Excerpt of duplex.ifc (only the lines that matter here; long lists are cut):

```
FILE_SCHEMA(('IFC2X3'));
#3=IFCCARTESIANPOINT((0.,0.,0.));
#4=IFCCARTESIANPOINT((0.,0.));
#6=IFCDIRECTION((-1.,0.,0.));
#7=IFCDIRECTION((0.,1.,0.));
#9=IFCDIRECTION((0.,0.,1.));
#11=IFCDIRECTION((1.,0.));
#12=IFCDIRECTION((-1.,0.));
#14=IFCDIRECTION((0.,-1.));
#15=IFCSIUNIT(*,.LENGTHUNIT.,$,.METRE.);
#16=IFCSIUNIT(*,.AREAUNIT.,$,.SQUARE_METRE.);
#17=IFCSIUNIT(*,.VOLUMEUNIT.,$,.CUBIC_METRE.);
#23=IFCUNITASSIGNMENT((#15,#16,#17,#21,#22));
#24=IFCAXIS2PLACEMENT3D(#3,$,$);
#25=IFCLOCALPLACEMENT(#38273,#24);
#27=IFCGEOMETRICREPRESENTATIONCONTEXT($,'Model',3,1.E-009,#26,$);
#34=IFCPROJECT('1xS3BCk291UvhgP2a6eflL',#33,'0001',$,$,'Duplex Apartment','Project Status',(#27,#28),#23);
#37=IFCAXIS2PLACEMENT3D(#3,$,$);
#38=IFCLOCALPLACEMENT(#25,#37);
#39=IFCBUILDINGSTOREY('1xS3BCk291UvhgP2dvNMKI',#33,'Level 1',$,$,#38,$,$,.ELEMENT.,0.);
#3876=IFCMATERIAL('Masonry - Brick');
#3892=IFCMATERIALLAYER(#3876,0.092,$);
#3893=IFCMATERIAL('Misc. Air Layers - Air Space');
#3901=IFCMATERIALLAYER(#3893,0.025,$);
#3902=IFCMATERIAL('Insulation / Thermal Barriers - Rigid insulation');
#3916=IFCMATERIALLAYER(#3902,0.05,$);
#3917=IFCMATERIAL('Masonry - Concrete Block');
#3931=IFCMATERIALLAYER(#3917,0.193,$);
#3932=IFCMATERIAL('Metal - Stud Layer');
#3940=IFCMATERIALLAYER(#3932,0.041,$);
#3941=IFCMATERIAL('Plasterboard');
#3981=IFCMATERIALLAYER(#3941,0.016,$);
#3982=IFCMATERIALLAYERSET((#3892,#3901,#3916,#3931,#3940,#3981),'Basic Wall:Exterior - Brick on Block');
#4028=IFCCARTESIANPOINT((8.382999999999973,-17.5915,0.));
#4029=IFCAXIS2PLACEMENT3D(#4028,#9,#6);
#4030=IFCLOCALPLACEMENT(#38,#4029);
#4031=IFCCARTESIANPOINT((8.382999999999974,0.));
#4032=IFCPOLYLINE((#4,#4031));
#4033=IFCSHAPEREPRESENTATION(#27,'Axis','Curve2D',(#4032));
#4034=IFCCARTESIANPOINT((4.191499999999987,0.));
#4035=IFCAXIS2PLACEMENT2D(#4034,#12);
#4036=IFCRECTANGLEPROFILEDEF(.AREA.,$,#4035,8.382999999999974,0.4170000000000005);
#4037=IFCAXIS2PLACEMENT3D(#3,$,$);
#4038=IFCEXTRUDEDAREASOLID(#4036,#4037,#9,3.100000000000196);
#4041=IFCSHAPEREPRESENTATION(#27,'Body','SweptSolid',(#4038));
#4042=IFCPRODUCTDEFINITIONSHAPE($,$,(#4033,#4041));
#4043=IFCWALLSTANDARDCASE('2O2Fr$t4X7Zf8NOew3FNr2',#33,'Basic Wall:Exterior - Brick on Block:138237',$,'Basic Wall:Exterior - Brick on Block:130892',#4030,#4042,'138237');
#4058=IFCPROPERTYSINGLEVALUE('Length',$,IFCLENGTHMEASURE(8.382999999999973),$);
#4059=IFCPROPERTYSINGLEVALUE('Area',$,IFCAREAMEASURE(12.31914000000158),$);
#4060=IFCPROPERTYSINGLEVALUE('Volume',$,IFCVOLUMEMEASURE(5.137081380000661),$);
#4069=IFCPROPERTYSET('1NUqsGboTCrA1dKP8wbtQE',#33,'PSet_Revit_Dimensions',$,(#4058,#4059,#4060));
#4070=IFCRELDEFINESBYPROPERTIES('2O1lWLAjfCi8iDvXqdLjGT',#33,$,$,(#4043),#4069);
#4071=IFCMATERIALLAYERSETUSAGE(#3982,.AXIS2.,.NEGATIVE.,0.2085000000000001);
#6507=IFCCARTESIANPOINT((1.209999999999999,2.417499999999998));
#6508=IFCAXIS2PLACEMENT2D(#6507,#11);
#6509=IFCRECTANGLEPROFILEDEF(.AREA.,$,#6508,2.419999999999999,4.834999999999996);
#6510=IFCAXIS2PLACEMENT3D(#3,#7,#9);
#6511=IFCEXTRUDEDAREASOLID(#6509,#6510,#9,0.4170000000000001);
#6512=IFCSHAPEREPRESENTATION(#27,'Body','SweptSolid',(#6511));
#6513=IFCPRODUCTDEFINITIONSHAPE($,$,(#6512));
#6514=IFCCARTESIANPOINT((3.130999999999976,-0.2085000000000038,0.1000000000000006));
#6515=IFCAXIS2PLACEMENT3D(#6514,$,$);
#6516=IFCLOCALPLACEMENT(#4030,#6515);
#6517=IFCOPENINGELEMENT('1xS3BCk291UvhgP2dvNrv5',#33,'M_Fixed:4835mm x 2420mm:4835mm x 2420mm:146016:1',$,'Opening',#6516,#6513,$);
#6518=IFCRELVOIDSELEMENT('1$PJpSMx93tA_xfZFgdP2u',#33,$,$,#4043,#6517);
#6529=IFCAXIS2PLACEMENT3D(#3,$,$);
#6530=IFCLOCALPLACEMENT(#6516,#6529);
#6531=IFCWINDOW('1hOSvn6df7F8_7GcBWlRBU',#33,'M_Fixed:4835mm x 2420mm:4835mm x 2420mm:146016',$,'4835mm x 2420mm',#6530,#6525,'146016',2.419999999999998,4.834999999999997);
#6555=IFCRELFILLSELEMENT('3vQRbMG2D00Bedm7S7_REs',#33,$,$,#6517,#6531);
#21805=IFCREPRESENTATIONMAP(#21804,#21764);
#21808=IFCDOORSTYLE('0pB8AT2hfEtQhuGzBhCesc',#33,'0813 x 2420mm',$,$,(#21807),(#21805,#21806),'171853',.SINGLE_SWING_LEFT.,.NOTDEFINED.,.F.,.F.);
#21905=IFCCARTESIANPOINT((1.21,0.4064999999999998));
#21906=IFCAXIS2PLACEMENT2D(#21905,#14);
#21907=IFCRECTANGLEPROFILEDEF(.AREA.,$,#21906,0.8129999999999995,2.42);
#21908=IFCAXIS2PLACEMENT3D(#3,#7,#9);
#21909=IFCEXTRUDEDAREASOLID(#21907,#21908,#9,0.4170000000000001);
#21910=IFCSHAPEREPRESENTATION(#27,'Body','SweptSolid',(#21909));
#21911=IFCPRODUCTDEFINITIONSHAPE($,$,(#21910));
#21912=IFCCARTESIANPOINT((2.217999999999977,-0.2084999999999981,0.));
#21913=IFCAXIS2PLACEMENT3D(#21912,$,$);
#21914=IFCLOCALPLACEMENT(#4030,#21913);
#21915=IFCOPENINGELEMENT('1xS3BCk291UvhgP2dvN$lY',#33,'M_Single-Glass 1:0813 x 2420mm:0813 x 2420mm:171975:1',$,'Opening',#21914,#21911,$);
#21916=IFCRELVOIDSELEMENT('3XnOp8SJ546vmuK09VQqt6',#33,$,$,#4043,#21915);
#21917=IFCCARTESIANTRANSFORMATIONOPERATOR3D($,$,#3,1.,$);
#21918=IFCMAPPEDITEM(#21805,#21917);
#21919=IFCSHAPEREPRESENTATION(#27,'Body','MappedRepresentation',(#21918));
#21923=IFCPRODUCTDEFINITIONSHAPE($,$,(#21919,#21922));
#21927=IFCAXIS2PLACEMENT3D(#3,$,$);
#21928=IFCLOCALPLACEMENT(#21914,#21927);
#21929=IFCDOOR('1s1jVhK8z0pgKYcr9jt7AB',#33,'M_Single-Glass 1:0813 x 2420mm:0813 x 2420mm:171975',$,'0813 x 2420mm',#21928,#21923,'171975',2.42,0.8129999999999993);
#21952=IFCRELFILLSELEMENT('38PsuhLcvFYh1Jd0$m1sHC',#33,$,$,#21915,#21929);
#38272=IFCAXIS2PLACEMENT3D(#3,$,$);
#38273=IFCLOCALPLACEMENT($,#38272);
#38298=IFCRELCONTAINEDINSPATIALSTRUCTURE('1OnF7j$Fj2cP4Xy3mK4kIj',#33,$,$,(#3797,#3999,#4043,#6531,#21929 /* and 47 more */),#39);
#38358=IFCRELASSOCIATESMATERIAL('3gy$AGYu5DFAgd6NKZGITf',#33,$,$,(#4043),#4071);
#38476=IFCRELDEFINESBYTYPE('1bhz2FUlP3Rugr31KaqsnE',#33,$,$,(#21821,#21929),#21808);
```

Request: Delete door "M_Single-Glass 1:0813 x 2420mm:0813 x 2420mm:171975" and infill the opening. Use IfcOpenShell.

```python
import ifcopenshell
import ifcopenshell.api.feature
import ifcopenshell.api.pset
import ifcopenshell.api.root
import ifcopenshell.geom
import ifcopenshell.util.element
import ifcopenshell.util.shape
import ifcopenshell.util.unit

model = ifcopenshell.open("duplex.ifc")
area_scale = ifcopenshell.util.unit.calculate_unit_scale(model, "AREAUNIT")
volume_scale = ifcopenshell.util.unit.calculate_unit_scale(model, "VOLUMEUNIT")
settings = ifcopenshell.geom.settings()


def volume(element):
    """Net volume in cubic metres, openings subtracted."""
    shape = ifcopenshell.geom.create_shape(settings, element)
    return ifcopenshell.util.shape.get_volume(shape.geometry)


door = model.by_id(21929)
opening = door.FillsVoids[0].RelatingOpeningElement
wall = opening.VoidsElements[0].RelatingBuildingElement
before = volume(wall)

ifcopenshell.api.root.remove_product(model, product=door)
ifcopenshell.api.feature.remove_feature(model, feature=opening)

after = volume(wall)
thickness = 0.417  # wall thickness in metres

# Update the wall's stored quantities.
pset = model.by_id(ifcopenshell.util.element.get_pset(wall, "PSet_Revit_Dimensions", should_inherit=False)["id"])
ifcopenshell.api.pset.edit_pset(model, pset=pset, properties={
    "Area": model.create_entity("IfcAreaMeasure", after / thickness / area_scale),
    "Volume": model.create_entity("IfcVolumeMeasure", after / volume_scale),
})

print(f"wall volume {before:.3f} -> {after:.3f} m3")

model.write("duplex_edited.ifc")
```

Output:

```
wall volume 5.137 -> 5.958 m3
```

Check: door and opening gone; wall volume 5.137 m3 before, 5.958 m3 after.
